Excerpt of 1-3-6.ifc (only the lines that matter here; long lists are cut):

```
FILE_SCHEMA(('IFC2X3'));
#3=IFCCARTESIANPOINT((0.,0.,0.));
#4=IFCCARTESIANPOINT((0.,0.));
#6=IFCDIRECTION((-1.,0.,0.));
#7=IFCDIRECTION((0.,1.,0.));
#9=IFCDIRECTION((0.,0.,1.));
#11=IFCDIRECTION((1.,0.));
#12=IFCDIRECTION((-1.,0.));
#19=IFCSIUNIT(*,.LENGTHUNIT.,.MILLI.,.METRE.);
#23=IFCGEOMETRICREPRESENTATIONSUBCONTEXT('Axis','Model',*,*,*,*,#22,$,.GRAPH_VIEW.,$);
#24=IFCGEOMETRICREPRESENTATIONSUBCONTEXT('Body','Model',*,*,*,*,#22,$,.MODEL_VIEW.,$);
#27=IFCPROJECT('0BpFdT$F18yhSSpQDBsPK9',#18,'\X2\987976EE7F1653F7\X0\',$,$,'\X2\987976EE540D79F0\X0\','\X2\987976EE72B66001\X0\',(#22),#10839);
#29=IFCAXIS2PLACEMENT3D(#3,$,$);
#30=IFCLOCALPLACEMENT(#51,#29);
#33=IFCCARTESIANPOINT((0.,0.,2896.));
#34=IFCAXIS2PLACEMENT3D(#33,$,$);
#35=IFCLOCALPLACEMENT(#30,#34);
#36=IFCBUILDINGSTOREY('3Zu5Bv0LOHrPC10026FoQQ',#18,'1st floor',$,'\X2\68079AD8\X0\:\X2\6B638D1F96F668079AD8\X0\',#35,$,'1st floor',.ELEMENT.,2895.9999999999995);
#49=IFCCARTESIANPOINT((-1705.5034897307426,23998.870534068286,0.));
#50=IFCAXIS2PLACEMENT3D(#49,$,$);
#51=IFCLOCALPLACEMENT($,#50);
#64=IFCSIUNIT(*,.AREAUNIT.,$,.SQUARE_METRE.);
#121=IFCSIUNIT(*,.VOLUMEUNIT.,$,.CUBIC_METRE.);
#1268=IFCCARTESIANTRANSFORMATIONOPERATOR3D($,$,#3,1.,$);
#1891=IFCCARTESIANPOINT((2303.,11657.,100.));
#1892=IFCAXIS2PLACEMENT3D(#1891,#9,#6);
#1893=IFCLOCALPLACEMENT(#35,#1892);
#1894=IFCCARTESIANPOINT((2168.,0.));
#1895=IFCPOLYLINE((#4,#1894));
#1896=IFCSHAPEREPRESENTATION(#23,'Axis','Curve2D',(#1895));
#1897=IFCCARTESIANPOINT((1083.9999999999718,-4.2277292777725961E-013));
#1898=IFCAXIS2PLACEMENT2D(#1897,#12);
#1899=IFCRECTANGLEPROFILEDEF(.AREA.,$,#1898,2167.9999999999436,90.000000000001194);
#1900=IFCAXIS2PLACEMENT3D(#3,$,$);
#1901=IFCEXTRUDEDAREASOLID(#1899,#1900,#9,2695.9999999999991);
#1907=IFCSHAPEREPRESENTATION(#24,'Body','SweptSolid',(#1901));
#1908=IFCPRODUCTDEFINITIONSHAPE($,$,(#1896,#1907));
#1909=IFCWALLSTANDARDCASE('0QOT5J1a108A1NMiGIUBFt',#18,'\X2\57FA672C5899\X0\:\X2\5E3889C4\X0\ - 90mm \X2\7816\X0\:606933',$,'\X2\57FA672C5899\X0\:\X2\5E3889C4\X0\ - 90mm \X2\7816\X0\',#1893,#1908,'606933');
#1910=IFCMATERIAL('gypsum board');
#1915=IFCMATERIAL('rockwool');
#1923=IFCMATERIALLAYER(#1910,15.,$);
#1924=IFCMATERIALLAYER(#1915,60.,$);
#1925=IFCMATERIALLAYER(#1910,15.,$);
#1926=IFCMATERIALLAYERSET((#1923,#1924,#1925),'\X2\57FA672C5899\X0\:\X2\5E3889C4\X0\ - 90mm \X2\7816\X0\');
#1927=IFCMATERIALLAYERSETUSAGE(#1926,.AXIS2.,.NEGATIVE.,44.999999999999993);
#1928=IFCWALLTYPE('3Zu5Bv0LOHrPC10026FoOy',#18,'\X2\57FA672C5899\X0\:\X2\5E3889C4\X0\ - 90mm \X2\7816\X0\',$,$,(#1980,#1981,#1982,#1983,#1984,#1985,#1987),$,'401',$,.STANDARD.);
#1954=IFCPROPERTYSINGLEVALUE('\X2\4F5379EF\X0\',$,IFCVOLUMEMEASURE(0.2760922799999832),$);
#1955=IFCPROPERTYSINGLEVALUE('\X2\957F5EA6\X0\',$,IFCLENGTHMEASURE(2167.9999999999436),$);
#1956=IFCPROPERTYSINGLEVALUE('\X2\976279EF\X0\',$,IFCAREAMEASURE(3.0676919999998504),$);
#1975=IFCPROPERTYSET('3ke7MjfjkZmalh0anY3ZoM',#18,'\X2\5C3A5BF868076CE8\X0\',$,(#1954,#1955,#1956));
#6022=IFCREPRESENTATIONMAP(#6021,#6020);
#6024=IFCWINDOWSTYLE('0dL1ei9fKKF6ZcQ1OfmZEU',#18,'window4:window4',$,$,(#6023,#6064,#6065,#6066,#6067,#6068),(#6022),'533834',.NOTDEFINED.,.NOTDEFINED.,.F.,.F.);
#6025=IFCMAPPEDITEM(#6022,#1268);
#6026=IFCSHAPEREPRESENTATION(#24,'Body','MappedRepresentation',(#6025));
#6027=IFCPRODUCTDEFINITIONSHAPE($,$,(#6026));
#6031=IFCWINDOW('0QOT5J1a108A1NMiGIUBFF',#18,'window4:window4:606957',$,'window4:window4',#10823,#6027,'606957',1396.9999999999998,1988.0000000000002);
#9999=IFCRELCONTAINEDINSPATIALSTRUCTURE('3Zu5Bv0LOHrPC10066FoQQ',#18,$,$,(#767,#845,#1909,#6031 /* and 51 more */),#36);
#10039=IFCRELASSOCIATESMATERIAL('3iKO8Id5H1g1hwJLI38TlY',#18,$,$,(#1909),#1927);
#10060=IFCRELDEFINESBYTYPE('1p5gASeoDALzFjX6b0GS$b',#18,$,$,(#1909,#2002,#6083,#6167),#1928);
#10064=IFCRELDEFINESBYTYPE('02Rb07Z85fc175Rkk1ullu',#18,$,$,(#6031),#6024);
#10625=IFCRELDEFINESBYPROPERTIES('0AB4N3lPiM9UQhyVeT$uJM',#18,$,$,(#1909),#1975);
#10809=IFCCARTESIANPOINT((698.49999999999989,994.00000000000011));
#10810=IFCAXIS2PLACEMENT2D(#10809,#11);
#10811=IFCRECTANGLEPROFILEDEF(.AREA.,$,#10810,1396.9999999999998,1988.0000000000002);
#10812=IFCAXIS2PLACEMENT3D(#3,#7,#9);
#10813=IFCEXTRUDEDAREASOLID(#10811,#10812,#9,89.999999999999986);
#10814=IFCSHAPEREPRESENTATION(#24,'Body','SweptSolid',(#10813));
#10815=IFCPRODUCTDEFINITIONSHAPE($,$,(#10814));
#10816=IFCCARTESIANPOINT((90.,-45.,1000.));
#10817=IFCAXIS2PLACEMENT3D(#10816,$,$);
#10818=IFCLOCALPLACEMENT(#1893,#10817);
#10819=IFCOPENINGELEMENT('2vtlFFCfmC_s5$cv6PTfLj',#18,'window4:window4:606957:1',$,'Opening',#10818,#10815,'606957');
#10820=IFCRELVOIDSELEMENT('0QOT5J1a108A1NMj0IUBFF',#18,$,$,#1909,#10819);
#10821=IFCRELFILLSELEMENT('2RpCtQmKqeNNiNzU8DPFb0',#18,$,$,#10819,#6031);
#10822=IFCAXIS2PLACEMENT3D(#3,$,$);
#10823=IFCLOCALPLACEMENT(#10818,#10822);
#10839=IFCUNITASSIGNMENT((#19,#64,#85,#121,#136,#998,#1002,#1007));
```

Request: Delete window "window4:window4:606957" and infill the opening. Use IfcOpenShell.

```python
import ifcopenshell
import ifcopenshell.api.feature
import ifcopenshell.api.pset
import ifcopenshell.api.root
import ifcopenshell.geom
import ifcopenshell.util.element
import ifcopenshell.util.shape
import ifcopenshell.util.unit

model = ifcopenshell.open("1-3-6.ifc")
area_scale = ifcopenshell.util.unit.calculate_unit_scale(model, "AREAUNIT")
volume_scale = ifcopenshell.util.unit.calculate_unit_scale(model, "VOLUMEUNIT")
settings = ifcopenshell.geom.settings()


def volume(element):
    """Net volume in cubic metres, openings subtracted."""
    shape = ifcopenshell.geom.create_shape(settings, element)
    return ifcopenshell.util.shape.get_volume(shape.geometry)


window = model.by_guid("0QOT5J1a108A1NMiGIUBFF")
opening = window.FillsVoids[0].RelatingOpeningElement
wall = opening.VoidsElements[0].RelatingBuildingElement
before = volume(wall)

ifcopenshell.api.root.remove_product(model, product=window)
ifcopenshell.api.feature.remove_feature(model, feature=opening)

after = volume(wall)
thickness = 0.09  # wall thickness in metres

# Update the wall's stored quantities.
pset = model.by_id(ifcopenshell.util.element.get_pset(wall, "尺寸标注", should_inherit=False)["id"])
ifcopenshell.api.pset.edit_pset(model, pset=pset, properties={
    "体积": model.create_entity("IfcVolumeMeasure", after / volume_scale),
    "面积": model.create_entity("IfcAreaMeasure", after / thickness / area_scale),
})

print(f"wall volume {before:.3f} -> {after:.3f} m3")

model.write("1-3-6_v2.ifc")
```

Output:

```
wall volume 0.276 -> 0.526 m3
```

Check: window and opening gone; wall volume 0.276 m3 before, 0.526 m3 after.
